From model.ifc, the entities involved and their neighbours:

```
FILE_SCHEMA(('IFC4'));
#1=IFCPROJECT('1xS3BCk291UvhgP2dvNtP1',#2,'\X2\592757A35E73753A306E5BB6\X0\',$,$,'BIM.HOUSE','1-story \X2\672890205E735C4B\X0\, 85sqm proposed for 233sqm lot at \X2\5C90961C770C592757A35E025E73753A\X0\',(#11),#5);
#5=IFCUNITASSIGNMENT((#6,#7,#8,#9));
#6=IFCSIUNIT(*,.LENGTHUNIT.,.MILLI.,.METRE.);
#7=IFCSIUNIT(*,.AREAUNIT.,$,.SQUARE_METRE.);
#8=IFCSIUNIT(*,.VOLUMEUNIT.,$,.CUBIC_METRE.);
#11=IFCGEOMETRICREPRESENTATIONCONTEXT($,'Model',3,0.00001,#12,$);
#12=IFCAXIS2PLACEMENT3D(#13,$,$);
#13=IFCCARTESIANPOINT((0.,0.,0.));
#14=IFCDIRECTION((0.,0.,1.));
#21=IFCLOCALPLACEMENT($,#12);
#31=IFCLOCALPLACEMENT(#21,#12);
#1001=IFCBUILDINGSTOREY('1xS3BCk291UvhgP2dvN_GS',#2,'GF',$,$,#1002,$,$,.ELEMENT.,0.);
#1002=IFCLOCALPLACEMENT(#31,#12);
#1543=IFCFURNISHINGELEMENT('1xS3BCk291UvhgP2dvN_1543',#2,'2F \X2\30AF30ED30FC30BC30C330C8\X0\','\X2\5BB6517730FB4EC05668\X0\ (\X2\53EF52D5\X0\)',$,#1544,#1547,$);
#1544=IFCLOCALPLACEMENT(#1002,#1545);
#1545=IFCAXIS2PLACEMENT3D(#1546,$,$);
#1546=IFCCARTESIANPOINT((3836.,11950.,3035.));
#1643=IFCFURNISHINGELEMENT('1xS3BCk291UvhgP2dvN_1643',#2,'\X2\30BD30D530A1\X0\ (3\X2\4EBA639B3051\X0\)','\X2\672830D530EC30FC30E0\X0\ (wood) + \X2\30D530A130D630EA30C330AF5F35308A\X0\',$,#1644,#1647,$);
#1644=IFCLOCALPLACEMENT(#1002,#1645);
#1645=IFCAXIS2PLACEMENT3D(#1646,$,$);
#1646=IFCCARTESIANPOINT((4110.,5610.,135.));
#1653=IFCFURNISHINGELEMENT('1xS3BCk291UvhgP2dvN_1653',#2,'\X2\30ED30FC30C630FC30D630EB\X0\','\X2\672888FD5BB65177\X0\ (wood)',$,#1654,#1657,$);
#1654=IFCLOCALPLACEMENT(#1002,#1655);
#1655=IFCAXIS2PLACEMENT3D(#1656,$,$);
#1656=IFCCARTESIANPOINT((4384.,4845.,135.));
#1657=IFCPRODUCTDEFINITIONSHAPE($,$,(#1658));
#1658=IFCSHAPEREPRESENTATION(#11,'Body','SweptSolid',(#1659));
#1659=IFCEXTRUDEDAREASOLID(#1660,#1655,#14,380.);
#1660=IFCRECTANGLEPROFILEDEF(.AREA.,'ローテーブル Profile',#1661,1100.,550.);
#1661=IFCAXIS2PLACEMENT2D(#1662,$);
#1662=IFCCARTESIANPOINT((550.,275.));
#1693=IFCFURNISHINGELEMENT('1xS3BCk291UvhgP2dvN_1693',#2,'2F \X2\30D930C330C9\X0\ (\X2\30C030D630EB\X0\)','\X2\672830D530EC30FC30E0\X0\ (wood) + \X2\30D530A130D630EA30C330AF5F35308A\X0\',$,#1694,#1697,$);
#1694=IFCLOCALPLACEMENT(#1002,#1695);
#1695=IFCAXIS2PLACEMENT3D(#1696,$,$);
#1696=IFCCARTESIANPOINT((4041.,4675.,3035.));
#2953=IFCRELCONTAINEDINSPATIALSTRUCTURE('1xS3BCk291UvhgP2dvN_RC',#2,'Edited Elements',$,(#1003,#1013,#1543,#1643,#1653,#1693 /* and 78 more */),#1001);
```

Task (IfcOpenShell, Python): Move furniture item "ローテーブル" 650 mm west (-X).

```python
import ifcopenshell
import ifcopenshell.api.geometry
import ifcopenshell.util.placement
import ifcopenshell.util.unit

model = ifcopenshell.open("model.ifc")
unit_scale = ifcopenshell.util.unit.calculate_unit_scale(model)

item = model.by_guid("1xS3BCk291UvhgP2dvN_1653")
matrix = ifcopenshell.util.placement.get_local_placement(item.ObjectPlacement)
matrix[0, 3] -= 0.65 / unit_scale
ifcopenshell.api.geometry.edit_object_placement(model, product=item, matrix=matrix, is_si=False)

print(ifcopenshell.util.placement.get_local_placement(item.ObjectPlacement).round(3) + 0.0)

model.write("model_updated.ifc")
```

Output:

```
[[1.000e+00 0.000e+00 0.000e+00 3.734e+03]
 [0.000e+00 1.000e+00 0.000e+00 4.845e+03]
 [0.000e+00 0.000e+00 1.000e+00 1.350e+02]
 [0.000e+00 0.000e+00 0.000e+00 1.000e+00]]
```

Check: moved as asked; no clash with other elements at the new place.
